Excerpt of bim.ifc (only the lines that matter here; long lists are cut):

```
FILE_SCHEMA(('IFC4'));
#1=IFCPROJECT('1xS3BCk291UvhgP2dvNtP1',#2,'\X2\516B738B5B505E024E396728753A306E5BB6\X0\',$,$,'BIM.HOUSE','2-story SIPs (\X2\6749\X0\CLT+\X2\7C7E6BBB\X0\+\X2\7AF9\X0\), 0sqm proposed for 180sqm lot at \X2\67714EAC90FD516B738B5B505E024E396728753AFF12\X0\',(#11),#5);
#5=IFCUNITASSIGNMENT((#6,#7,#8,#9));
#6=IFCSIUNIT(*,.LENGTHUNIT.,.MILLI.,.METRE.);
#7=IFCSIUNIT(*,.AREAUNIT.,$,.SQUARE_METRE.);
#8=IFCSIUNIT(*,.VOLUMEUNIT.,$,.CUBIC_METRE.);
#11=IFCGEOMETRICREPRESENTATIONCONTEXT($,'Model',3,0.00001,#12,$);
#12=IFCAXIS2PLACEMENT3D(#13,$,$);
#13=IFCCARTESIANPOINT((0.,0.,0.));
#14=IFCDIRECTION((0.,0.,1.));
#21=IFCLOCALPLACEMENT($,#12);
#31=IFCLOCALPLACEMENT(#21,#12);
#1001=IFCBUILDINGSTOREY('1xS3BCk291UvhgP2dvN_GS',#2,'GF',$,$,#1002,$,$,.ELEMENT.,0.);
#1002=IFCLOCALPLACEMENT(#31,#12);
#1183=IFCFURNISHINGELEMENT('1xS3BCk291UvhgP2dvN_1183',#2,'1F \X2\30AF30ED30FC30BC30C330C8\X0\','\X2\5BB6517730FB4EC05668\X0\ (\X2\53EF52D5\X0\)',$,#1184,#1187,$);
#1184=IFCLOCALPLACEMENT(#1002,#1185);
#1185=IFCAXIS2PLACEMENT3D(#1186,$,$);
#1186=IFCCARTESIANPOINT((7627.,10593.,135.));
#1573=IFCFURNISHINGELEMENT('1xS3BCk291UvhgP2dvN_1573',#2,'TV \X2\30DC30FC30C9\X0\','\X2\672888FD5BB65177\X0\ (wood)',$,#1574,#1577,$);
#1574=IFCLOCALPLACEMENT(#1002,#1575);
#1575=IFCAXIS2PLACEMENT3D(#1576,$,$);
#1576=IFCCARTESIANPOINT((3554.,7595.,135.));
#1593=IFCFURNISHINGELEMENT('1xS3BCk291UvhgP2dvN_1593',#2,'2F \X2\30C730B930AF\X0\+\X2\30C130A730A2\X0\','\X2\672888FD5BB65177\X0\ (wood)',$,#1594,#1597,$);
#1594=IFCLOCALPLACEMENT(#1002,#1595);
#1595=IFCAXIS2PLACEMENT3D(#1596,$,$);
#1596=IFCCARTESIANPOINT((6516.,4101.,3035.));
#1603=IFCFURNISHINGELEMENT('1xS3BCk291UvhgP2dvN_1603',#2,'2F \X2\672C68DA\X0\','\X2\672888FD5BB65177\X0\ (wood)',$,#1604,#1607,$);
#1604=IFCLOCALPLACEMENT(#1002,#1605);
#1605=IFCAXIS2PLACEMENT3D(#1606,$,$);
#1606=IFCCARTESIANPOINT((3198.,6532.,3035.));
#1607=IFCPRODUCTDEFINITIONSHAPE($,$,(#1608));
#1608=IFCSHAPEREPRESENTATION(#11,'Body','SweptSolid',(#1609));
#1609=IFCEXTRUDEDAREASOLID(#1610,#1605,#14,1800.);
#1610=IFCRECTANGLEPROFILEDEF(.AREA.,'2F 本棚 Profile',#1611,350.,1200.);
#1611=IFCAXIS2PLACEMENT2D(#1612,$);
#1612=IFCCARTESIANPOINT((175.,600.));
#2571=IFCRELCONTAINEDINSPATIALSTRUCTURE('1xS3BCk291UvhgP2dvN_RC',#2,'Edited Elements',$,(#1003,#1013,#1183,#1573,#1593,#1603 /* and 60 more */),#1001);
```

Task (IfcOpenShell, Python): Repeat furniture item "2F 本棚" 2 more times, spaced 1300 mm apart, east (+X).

```python
import numpy as np
import ifcopenshell
import ifcopenshell.api.geometry
import ifcopenshell.api.root
import ifcopenshell.util.element
import ifcopenshell.util.placement
import ifcopenshell.util.unit

model = ifcopenshell.open("bim.ifc")
unit_scale = ifcopenshell.util.unit.calculate_unit_scale(model)


def reuse_history(source, copy):
    """copy_class also copies each property set's owner history, people and application; keep the originals."""
    for rel in copy.IsDefinedBy:
        if rel.is_a("IfcRelDefinesByProperties") and (history := rel.RelatingPropertyDefinition.OwnerHistory):
            rel.RelatingPropertyDefinition.OwnerHistory = source.OwnerHistory
            ifcopenshell.util.element.remove_deep2(model, history)


source = model.by_guid("1xS3BCk291UvhgP2dvN_1603")
base = ifcopenshell.util.placement.get_local_placement(source.ObjectPlacement)
step = np.array([1.0, 0.0, 0.0]) * 1.3 / unit_scale

for i in range(1, 3):
    copy = ifcopenshell.api.root.copy_class(model, product=source)
    copy.Representation = ifcopenshell.util.element.copy_deep(
        model, source.Representation, exclude=["IfcGeometricRepresentationContext", "IfcRepresentationMap"]
    )
    reuse_history(source, copy)
    matrix = base.copy()
    matrix[:3, 3] += i * step
    print("added at", matrix[:3, 3].round(3) + 0.0)
    ifcopenshell.api.geometry.edit_object_placement(model, product=copy, matrix=matrix, is_si=False)

model.write("bim_rev.ifc")
```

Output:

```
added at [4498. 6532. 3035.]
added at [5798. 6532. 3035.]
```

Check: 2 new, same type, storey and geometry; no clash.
